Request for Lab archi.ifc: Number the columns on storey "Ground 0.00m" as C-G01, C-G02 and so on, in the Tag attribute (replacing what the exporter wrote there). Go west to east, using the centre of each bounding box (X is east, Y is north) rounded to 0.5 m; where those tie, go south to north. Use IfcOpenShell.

First a look at what the model holds.

```python
import ifcopenshell
import ifcopenshell.util.element
import ifcopenshell.util.placement

model = ifcopenshell.open("Lab archi.ifc")
print(model.schema)
storey = next(s for s in model.by_type("IfcBuildingStorey") if s.Name == "Ground 0.00m")
columns = [e for e in ifcopenshell.util.element.get_decomposition(storey) if e.is_a("IfcColumn")]
for e in sorted(columns, key=lambda e: e.id()):
    origin = ifcopenshell.util.placement.get_local_placement(e.ObjectPlacement)[:3, 3]
    print(e.id(), e.Tag, e.Name, origin.round(2) + 0.0, sep=" | ")
```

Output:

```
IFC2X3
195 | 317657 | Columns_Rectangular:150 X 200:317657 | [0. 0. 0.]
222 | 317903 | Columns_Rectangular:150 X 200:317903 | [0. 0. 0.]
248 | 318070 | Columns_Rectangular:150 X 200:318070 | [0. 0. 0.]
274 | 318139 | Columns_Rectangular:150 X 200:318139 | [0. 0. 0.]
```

```python
import ifcopenshell
import ifcopenshell.geom
import ifcopenshell.util.element
import ifcopenshell.util.shape

model = ifcopenshell.open("Lab archi.ifc")
settings = ifcopenshell.geom.settings()
settings.set("use-world-coords", True)


def centre(element):
    shape = ifcopenshell.geom.create_shape(settings, element)
    return ifcopenshell.util.shape.get_bbox_centroid(shape.geometry)


storey = next(s for s in model.by_type("IfcBuildingStorey") if s.Name == "Ground 0.00m")
columns = [e for e in ifcopenshell.util.element.get_decomposition(storey) if e.is_a("IfcColumn")]

# Insertion points can sit at a corner or the storey origin, so sort by the geometry (in metres).
centres = {e: centre(e) for e in columns}
columns.sort(key=lambda e: (round(centres[e][0] / 0.5), centres[e][1]))

for i, e in enumerate(columns, start=1):
    number = f"C-G{i:02d}"
    e.Tag = number
    print(e.id(), number)

model.write("Lab archi_rev.ifc")
```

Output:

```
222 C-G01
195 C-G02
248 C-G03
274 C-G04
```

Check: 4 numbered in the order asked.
